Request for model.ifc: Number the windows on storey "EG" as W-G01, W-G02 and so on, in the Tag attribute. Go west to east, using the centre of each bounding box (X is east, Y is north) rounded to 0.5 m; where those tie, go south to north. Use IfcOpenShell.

First a look at what the model holds.

```python
import ifcopenshell
import ifcopenshell.util.element
import ifcopenshell.util.placement

model = ifcopenshell.open("model.ifc")
print(model.schema)
storey = next(s for s in model.by_type("IfcBuildingStorey") if s.Name == "EG")
windows = [e for e in ifcopenshell.util.element.get_decomposition(storey) if e.is_a("IfcWindow")]
for e in sorted(windows, key=lambda e: e.id()):
    origin = ifcopenshell.util.placement.get_local_placement(e.ObjectPlacement)[:3, 3]
    print(e.id(), e.Tag, e.Name, origin.round(2) + 0.0, sep=" | ")
```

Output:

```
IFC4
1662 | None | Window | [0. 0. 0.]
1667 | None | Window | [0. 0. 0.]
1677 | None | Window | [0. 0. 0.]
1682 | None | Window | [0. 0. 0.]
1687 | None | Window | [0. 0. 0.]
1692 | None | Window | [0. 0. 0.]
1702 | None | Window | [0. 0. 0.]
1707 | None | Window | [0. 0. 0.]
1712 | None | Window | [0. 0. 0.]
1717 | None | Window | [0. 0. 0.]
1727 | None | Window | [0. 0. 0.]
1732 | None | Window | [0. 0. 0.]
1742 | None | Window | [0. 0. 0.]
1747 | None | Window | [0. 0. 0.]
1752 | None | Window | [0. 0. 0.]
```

```python
import ifcopenshell
import ifcopenshell.geom
import ifcopenshell.util.element
import ifcopenshell.util.shape

model = ifcopenshell.open("model.ifc")
settings = ifcopenshell.geom.settings()
settings.set("use-world-coords", True)


def centre(element):
    shape = ifcopenshell.geom.create_shape(settings, element)
    return ifcopenshell.util.shape.get_bbox_centroid(shape.geometry)


storey = next(s for s in model.by_type("IfcBuildingStorey") if s.Name == "EG")
windows = [e for e in ifcopenshell.util.element.get_decomposition(storey) if e.is_a("IfcWindow")]

# Insertion points can sit at a corner or the storey origin, so sort by the geometry (in metres).
centres = {e: centre(e) for e in windows}
windows.sort(key=lambda e: (round(centres[e][0] / 0.5), centres[e][1]))

for i, e in enumerate(windows, start=1):
    number = f"W-G{i:02d}"
    e.Tag = number
    print(e.id(), number)

model.write("model_rev.ifc")
```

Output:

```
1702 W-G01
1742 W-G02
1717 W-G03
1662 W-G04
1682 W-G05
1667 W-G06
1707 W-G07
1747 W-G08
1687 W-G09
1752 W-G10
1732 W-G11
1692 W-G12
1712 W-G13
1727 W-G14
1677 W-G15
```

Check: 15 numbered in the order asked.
